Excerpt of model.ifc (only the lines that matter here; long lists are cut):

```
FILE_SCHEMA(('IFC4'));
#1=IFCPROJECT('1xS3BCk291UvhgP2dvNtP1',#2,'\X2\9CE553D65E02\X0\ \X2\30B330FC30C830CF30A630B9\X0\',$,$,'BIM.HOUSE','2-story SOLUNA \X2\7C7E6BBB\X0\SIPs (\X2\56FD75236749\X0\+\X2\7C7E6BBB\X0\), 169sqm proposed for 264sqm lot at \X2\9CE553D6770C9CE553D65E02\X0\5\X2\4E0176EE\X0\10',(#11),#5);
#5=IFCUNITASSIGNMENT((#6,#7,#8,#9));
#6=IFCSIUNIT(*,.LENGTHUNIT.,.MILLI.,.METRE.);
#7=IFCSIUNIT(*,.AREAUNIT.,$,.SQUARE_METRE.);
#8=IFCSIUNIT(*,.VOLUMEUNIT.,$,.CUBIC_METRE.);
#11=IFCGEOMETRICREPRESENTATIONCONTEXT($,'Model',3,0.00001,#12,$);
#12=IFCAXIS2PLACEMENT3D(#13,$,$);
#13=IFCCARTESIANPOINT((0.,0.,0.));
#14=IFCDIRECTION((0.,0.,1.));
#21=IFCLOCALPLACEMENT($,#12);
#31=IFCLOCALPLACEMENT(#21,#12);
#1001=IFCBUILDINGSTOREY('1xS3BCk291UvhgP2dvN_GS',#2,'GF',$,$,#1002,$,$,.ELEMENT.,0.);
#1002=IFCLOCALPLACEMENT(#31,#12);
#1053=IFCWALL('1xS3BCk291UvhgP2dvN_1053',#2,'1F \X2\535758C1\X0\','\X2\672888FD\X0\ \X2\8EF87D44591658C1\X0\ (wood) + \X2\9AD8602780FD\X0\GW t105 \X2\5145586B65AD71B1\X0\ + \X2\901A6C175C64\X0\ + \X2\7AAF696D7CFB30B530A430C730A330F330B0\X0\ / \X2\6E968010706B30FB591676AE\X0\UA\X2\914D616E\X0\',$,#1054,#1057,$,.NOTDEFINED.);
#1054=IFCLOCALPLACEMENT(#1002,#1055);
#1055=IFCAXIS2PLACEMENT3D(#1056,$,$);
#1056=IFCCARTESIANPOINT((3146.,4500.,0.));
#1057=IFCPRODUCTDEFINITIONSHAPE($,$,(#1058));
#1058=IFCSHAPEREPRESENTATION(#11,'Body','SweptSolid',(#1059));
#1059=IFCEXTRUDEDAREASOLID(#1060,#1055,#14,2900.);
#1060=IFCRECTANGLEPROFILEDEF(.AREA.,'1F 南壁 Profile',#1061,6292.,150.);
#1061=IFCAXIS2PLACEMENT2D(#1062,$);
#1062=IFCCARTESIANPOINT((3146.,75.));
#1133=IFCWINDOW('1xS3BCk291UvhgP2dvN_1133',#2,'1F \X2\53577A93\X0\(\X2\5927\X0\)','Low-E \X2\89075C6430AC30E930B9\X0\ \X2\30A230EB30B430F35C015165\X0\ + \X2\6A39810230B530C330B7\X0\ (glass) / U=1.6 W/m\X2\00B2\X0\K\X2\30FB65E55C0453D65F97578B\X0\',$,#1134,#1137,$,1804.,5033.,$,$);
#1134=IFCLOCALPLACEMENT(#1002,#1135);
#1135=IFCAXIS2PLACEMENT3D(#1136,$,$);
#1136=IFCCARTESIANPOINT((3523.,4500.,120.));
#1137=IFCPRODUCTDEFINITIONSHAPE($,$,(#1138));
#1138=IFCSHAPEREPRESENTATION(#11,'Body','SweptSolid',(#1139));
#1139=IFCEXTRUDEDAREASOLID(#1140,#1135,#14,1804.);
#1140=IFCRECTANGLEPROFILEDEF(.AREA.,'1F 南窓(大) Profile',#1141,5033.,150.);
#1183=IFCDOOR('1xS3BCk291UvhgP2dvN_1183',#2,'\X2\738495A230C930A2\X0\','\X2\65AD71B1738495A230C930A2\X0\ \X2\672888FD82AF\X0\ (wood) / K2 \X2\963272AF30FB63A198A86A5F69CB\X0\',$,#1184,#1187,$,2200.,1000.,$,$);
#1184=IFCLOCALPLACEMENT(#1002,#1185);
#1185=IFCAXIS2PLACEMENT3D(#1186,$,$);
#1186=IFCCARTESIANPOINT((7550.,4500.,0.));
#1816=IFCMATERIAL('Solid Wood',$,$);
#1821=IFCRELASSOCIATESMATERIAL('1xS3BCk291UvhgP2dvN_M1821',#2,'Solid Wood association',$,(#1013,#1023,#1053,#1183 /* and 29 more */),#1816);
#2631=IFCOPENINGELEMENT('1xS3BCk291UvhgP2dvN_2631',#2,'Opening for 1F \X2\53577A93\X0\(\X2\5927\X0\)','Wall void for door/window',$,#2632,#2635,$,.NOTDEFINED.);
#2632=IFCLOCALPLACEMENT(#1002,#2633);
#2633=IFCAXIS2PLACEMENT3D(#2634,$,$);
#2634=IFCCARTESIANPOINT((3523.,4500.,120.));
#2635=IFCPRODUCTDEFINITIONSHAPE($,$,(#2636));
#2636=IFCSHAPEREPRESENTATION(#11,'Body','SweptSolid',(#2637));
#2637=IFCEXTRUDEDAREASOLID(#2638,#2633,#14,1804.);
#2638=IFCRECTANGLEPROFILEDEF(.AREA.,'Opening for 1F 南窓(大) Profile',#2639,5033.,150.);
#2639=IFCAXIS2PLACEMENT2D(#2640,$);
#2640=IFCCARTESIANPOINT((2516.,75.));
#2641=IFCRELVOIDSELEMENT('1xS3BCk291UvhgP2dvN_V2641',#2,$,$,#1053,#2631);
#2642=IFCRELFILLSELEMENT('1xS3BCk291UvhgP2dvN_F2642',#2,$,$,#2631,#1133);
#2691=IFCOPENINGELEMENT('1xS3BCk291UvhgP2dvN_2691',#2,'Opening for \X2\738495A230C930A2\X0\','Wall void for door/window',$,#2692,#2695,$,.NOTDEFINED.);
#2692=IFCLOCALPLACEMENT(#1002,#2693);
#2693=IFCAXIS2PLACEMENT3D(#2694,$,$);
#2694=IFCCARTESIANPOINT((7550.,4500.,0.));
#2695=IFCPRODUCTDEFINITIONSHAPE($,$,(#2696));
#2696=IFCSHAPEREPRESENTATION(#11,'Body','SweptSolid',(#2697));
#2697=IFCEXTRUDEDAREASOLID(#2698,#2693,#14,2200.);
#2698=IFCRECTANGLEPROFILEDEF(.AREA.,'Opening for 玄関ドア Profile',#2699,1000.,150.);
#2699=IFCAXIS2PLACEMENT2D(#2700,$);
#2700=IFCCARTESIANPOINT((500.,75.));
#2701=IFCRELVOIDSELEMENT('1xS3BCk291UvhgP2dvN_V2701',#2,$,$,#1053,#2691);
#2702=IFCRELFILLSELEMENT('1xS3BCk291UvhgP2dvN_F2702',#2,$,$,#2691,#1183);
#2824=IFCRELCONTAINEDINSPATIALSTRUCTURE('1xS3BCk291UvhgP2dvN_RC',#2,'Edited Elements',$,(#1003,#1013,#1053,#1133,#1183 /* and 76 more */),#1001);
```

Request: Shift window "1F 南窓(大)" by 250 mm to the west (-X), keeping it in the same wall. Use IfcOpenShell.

```python
import ifcopenshell
import ifcopenshell.api.geometry
import ifcopenshell.util.placement
import ifcopenshell.util.unit

model = ifcopenshell.open("model.ifc")
unit_scale = ifcopenshell.util.unit.calculate_unit_scale(model)

window = model.by_id(1133)
opening = window.FillsVoids[0].RelatingOpeningElement
wall = opening.VoidsElements[0].RelatingBuildingElement

wall_matrix = ifcopenshell.util.placement.get_local_placement(wall.ObjectPlacement)
shift = wall_matrix[:3, 0] * -0.25 / unit_scale
before = ifcopenshell.util.placement.get_local_placement(window.ObjectPlacement)[:3, 3].copy()

# The window is not placed relative to its opening, so move both.
for product in (opening, window):
    matrix = ifcopenshell.util.placement.get_local_placement(product.ObjectPlacement)
    matrix[:3, 3] += shift
    ifcopenshell.api.geometry.edit_object_placement(model, product=product, matrix=matrix, is_si=False)

after = ifcopenshell.util.placement.get_local_placement(window.ObjectPlacement)[:3, 3]
print("window moved by", (after - before).round(3) + 0.0)

model.write("model_edited.ifc")
```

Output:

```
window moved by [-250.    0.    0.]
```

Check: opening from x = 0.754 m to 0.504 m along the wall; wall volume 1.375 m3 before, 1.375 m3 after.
